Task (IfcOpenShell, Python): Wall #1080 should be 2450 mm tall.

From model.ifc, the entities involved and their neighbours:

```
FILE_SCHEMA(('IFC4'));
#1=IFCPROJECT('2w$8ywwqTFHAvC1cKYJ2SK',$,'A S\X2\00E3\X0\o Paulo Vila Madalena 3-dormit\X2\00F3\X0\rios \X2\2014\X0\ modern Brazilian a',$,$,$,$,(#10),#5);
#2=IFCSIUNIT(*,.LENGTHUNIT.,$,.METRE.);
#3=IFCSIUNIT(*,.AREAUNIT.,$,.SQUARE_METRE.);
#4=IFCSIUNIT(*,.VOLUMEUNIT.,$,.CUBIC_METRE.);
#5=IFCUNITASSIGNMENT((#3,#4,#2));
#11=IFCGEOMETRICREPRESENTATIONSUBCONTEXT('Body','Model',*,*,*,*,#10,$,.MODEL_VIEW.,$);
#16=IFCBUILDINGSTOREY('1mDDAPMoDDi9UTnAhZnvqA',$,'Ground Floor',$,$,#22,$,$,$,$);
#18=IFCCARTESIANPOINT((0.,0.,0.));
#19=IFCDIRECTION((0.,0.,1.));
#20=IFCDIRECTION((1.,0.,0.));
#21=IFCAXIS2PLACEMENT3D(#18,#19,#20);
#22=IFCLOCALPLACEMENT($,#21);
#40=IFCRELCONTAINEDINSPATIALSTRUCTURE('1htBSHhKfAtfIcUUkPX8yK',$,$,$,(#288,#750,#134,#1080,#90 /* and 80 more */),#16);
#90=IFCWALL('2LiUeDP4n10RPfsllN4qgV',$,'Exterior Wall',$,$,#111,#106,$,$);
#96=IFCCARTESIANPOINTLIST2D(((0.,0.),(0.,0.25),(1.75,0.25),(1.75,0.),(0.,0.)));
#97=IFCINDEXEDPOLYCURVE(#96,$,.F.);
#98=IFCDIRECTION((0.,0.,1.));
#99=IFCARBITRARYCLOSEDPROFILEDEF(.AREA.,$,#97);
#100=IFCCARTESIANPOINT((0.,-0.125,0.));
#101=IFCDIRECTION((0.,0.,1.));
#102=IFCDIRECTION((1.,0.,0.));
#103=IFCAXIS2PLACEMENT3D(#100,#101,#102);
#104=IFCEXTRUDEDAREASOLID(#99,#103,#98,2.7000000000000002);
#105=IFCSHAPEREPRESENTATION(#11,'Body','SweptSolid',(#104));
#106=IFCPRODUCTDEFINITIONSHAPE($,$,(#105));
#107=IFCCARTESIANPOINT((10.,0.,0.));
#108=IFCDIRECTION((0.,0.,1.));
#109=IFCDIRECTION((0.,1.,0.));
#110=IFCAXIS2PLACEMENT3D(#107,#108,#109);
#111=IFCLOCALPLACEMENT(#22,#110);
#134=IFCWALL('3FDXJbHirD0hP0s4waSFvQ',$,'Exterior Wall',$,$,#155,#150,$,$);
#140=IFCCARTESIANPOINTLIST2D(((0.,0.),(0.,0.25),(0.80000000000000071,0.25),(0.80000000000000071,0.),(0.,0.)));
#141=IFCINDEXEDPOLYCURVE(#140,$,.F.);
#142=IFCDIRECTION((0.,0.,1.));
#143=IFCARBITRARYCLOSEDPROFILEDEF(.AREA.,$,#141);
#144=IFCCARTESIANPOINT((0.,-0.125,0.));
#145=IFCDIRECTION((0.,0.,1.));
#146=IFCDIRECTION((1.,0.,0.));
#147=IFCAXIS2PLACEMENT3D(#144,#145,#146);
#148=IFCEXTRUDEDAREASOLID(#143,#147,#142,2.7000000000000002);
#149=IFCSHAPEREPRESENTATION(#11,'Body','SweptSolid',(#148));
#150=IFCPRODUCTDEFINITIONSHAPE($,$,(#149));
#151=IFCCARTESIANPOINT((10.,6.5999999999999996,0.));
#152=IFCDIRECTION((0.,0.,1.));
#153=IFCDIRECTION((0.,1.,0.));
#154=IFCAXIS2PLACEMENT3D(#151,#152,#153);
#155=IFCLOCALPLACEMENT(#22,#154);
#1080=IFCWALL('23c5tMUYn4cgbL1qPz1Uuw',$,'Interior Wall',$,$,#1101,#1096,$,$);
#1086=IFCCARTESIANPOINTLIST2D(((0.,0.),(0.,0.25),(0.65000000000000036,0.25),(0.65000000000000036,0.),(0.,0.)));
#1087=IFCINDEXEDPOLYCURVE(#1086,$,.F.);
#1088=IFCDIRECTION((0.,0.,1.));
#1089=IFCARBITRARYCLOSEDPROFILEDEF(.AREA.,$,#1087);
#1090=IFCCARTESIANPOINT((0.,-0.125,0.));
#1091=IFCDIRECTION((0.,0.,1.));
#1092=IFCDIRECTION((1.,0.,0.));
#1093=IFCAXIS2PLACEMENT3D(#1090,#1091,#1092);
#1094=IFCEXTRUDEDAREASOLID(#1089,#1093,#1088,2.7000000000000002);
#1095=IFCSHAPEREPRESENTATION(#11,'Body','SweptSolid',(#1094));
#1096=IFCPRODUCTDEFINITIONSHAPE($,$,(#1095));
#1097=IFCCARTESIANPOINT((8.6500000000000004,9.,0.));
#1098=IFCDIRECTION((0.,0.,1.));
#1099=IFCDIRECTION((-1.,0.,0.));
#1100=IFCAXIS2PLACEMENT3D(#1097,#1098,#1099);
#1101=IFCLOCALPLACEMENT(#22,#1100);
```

```python
import ifcopenshell
import ifcopenshell.geom
import ifcopenshell.util.representation
import ifcopenshell.util.shape
import ifcopenshell.util.unit

model = ifcopenshell.open("model.ifc")
unit_scale = ifcopenshell.util.unit.calculate_unit_scale(model)
settings = ifcopenshell.geom.settings()


def volume(element):
    """Net volume in cubic metres, openings subtracted."""
    shape = ifcopenshell.geom.create_shape(settings, element)
    return ifcopenshell.util.shape.get_volume(shape.geometry)


wall = model.by_guid("23c5tMUYn4cgbL1qPz1Uuw")
before = volume(wall)

body = ifcopenshell.util.representation.get_representation(wall, "Model", "Body")
solid = body.Items[0]
old_height = solid.Depth
solid.Depth = 2.45 / unit_scale
after = volume(wall)

print(f"height {old_height:g} -> {solid.Depth:g}, volume {before:.3f} -> {after:.3f} m3")

model.write("model_edited.ifc")
```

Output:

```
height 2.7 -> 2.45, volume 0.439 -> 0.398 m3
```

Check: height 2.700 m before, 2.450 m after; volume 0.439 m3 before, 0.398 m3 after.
